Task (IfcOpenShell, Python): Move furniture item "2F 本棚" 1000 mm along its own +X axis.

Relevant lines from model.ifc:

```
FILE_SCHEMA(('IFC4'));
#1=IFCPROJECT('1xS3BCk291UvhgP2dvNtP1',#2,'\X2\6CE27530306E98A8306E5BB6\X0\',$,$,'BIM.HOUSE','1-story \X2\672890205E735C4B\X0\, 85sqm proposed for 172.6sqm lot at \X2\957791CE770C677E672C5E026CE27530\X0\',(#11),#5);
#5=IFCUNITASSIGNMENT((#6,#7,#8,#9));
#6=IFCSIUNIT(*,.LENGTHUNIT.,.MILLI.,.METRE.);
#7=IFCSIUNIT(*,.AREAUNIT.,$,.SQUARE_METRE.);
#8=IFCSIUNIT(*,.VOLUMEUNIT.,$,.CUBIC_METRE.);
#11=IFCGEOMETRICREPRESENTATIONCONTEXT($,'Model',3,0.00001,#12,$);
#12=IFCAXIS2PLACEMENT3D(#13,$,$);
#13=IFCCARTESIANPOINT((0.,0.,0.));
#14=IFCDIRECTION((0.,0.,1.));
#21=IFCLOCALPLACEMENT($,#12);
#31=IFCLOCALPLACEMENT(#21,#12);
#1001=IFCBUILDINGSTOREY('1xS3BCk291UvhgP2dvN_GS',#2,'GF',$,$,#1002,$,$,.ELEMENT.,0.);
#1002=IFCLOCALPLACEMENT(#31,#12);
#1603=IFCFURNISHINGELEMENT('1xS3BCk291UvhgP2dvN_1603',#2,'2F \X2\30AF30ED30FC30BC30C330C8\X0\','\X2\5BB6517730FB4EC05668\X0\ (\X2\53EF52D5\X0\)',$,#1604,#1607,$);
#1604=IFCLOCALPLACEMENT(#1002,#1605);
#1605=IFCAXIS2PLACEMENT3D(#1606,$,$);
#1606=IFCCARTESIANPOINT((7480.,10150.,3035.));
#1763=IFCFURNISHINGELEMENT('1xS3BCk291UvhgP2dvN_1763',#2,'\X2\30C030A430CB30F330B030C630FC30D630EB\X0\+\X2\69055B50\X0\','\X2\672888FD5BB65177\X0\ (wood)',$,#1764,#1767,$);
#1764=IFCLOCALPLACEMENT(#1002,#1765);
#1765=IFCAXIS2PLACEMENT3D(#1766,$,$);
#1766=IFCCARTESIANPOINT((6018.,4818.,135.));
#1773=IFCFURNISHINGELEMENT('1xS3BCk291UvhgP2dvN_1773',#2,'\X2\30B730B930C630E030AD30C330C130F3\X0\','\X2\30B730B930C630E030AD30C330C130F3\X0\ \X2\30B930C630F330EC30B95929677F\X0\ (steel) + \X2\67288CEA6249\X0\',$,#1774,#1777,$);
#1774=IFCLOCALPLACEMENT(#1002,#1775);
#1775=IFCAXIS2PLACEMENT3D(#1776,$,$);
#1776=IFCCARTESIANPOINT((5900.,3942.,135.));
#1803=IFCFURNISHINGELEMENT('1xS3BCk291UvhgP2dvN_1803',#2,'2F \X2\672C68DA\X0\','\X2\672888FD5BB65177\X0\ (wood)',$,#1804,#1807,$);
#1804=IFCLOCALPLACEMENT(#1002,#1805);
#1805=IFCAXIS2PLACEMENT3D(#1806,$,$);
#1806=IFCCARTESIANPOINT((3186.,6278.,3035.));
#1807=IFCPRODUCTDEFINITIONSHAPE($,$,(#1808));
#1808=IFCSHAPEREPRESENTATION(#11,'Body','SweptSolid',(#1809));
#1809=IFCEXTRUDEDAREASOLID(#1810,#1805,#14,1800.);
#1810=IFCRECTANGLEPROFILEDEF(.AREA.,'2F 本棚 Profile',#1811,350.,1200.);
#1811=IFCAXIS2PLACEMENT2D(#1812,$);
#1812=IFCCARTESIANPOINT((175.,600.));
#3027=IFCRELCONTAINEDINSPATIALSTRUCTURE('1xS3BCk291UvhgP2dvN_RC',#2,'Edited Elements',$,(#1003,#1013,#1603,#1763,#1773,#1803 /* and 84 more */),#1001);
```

```python
import ifcopenshell
import ifcopenshell.api.geometry
import ifcopenshell.util.placement
import ifcopenshell.util.unit

model = ifcopenshell.open("model.ifc")
unit_scale = ifcopenshell.util.unit.calculate_unit_scale(model)

item = model.by_guid("1xS3BCk291UvhgP2dvN_1803")
matrix = ifcopenshell.util.placement.get_local_placement(item.ObjectPlacement)
matrix[:3, 3] += matrix[:3, 0] * 1 / unit_scale
ifcopenshell.api.geometry.edit_object_placement(model, product=item, matrix=matrix, is_si=False)

print(ifcopenshell.util.placement.get_local_placement(item.ObjectPlacement).round(3) + 0.0)

model.write("model_v2.ifc")
```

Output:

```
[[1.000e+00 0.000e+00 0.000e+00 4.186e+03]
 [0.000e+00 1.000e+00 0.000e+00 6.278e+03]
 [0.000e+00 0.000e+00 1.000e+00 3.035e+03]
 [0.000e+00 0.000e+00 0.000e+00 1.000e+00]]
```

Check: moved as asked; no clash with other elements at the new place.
